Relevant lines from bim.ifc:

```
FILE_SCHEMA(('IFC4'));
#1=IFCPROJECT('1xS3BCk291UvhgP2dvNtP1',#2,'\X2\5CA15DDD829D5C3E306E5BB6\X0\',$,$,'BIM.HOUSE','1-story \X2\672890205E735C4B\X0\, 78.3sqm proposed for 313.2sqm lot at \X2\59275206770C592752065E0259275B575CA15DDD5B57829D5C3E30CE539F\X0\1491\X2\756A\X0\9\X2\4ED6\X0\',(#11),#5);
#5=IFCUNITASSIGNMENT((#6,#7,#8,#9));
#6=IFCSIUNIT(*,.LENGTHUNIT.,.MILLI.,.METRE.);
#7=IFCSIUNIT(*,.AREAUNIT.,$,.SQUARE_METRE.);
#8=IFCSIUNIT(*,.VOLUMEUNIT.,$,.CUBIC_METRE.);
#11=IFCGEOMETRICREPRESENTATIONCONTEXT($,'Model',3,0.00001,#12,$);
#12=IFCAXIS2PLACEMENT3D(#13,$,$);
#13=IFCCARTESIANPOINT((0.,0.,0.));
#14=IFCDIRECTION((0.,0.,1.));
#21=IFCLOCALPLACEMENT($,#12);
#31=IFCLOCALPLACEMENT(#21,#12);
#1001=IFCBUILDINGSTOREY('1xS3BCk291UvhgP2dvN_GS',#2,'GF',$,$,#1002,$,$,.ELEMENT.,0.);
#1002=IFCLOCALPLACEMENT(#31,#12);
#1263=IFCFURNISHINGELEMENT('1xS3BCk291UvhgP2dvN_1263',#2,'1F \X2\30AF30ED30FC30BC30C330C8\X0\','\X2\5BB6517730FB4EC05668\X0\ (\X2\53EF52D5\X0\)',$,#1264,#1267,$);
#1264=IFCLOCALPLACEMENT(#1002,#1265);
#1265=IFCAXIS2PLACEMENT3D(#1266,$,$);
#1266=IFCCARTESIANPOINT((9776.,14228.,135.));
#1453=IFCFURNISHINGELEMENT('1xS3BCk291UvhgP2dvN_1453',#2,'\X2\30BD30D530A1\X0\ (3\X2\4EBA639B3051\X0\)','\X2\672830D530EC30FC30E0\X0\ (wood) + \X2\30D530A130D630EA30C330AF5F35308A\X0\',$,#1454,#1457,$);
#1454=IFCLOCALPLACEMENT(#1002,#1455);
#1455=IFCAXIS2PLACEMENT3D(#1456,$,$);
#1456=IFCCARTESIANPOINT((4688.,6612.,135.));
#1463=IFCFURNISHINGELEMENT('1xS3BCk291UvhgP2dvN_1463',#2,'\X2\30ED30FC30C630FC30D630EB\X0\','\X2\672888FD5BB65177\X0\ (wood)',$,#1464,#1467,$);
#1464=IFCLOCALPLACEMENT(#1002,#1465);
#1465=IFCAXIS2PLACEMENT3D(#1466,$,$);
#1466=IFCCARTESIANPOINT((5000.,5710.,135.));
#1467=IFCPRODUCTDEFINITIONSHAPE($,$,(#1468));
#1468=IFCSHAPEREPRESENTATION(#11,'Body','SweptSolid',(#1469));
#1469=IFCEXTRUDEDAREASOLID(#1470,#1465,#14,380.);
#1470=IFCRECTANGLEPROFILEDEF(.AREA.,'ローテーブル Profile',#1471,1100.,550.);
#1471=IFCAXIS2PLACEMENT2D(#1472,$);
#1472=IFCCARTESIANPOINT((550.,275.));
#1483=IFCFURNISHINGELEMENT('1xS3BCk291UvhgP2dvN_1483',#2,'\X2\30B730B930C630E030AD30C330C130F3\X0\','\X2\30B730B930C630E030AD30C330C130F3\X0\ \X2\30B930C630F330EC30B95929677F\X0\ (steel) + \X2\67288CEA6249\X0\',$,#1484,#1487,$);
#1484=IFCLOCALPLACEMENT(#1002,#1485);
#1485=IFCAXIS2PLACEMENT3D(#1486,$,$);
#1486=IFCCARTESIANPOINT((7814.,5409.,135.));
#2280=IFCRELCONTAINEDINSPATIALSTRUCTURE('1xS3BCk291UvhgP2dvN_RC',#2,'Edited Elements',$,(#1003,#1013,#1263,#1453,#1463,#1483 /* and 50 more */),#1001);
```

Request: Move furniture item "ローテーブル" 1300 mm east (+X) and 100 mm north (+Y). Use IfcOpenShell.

```python
import ifcopenshell
import ifcopenshell.api.geometry
import ifcopenshell.util.placement
import ifcopenshell.util.unit

model = ifcopenshell.open("bim.ifc")
unit_scale = ifcopenshell.util.unit.calculate_unit_scale(model)

item = model.by_guid("1xS3BCk291UvhgP2dvN_1463")
matrix = ifcopenshell.util.placement.get_local_placement(item.ObjectPlacement)
matrix[0, 3] += 1.3 / unit_scale
matrix[1, 3] += 0.1 / unit_scale
ifcopenshell.api.geometry.edit_object_placement(model, product=item, matrix=matrix, is_si=False)

print(ifcopenshell.util.placement.get_local_placement(item.ObjectPlacement).round(3) + 0.0)

model.write("bim_updated.ifc")
```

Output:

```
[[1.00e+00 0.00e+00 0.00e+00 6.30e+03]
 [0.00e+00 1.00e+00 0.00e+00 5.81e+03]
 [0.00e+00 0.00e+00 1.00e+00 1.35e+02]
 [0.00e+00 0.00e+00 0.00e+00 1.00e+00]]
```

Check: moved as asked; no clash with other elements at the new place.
